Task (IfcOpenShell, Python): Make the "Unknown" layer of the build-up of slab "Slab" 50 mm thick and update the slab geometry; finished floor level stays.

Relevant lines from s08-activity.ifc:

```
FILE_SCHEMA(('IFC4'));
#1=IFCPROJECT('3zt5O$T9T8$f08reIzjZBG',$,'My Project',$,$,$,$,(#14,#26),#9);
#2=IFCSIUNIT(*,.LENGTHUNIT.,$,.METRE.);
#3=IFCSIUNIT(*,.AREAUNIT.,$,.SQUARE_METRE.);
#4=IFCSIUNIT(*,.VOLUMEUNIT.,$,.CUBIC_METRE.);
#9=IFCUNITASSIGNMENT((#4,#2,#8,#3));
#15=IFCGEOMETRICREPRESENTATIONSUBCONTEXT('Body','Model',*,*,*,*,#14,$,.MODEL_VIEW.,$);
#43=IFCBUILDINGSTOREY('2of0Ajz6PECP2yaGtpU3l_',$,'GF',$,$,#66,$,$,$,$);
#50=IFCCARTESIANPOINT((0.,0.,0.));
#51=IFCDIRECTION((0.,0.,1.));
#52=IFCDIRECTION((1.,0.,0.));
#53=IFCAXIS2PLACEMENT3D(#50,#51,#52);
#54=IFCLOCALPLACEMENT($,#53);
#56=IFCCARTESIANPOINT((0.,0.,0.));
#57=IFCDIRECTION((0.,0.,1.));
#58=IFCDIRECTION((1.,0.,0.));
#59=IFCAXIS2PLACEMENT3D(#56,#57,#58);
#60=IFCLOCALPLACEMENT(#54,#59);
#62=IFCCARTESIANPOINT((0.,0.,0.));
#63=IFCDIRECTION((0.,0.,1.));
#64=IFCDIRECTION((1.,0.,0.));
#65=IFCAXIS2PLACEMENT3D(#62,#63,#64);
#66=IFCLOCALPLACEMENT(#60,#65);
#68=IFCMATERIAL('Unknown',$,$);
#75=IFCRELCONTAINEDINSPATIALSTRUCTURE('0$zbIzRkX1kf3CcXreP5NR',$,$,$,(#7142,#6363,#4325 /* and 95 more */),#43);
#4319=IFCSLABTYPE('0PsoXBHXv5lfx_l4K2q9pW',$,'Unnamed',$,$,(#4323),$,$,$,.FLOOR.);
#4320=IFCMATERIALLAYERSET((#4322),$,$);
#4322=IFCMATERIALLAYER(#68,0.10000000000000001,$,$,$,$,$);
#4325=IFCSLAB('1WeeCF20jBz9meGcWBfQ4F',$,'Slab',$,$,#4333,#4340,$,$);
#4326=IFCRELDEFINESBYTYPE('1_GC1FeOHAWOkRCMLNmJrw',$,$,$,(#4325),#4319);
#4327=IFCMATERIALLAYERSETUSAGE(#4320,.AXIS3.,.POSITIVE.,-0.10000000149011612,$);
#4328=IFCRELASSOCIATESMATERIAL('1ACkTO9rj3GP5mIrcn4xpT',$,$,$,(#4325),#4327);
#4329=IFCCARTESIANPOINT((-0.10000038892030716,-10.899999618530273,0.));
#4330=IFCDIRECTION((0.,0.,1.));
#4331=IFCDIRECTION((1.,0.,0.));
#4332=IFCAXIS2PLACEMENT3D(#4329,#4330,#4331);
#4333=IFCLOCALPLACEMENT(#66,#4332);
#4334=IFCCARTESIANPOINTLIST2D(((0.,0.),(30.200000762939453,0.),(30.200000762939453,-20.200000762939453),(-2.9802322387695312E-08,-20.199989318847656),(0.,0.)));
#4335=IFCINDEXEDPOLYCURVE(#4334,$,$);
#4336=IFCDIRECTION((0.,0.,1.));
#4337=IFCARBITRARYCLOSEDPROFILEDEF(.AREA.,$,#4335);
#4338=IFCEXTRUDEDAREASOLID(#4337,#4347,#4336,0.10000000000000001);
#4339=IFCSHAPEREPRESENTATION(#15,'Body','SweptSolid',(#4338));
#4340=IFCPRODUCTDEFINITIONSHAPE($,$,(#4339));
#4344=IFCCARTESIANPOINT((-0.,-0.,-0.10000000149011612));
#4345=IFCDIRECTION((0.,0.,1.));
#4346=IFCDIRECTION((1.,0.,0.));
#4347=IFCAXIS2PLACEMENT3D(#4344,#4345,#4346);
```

```python
import ifcopenshell
import ifcopenshell.util.element
import ifcopenshell.util.representation
import ifcopenshell.util.unit

model = ifcopenshell.open("s08-activity.ifc")
unit_scale = ifcopenshell.util.unit.calculate_unit_scale(model)

layer_set = model.by_id(4320)
layer = next(l for l in layer_set.MaterialLayers if l.Material and l.Material.Name == "Unknown")
change = 0.05 / unit_scale - layer.LayerThickness
layer.LayerThickness += change

# Geometry does not follow the layer set by itself.
slabs = [e for e in ifcopenshell.util.element.get_elements_by_material(model, layer_set) if e.is_a("IfcSlab")]
for slab in sorted(slabs, key=lambda e: e.id()):
    body = ifcopenshell.util.representation.get_representation(slab, "Model", "Body")
    solid = body.Items[0]
    old_depth = solid.Depth
    solid.Depth += change
    # Extruded upwards: lower the start of the extrusion so the top stays.
    x, y, z = solid.Position.Location.Coordinates
    solid.Position.Location = model.createIfcCartesianPoint((x, y, z - change))
    print(slab.id(), f"{old_depth:g} -> {solid.Depth:g}")

# The layers are counted up from the underside, which has moved.
for usage in {ifcopenshell.util.element.get_material(slab) for slab in slabs}:
    usage.OffsetFromReferenceLine -= change

model.write("s08-activity_updated.ifc")
```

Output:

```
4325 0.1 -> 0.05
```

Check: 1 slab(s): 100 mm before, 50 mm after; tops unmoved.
